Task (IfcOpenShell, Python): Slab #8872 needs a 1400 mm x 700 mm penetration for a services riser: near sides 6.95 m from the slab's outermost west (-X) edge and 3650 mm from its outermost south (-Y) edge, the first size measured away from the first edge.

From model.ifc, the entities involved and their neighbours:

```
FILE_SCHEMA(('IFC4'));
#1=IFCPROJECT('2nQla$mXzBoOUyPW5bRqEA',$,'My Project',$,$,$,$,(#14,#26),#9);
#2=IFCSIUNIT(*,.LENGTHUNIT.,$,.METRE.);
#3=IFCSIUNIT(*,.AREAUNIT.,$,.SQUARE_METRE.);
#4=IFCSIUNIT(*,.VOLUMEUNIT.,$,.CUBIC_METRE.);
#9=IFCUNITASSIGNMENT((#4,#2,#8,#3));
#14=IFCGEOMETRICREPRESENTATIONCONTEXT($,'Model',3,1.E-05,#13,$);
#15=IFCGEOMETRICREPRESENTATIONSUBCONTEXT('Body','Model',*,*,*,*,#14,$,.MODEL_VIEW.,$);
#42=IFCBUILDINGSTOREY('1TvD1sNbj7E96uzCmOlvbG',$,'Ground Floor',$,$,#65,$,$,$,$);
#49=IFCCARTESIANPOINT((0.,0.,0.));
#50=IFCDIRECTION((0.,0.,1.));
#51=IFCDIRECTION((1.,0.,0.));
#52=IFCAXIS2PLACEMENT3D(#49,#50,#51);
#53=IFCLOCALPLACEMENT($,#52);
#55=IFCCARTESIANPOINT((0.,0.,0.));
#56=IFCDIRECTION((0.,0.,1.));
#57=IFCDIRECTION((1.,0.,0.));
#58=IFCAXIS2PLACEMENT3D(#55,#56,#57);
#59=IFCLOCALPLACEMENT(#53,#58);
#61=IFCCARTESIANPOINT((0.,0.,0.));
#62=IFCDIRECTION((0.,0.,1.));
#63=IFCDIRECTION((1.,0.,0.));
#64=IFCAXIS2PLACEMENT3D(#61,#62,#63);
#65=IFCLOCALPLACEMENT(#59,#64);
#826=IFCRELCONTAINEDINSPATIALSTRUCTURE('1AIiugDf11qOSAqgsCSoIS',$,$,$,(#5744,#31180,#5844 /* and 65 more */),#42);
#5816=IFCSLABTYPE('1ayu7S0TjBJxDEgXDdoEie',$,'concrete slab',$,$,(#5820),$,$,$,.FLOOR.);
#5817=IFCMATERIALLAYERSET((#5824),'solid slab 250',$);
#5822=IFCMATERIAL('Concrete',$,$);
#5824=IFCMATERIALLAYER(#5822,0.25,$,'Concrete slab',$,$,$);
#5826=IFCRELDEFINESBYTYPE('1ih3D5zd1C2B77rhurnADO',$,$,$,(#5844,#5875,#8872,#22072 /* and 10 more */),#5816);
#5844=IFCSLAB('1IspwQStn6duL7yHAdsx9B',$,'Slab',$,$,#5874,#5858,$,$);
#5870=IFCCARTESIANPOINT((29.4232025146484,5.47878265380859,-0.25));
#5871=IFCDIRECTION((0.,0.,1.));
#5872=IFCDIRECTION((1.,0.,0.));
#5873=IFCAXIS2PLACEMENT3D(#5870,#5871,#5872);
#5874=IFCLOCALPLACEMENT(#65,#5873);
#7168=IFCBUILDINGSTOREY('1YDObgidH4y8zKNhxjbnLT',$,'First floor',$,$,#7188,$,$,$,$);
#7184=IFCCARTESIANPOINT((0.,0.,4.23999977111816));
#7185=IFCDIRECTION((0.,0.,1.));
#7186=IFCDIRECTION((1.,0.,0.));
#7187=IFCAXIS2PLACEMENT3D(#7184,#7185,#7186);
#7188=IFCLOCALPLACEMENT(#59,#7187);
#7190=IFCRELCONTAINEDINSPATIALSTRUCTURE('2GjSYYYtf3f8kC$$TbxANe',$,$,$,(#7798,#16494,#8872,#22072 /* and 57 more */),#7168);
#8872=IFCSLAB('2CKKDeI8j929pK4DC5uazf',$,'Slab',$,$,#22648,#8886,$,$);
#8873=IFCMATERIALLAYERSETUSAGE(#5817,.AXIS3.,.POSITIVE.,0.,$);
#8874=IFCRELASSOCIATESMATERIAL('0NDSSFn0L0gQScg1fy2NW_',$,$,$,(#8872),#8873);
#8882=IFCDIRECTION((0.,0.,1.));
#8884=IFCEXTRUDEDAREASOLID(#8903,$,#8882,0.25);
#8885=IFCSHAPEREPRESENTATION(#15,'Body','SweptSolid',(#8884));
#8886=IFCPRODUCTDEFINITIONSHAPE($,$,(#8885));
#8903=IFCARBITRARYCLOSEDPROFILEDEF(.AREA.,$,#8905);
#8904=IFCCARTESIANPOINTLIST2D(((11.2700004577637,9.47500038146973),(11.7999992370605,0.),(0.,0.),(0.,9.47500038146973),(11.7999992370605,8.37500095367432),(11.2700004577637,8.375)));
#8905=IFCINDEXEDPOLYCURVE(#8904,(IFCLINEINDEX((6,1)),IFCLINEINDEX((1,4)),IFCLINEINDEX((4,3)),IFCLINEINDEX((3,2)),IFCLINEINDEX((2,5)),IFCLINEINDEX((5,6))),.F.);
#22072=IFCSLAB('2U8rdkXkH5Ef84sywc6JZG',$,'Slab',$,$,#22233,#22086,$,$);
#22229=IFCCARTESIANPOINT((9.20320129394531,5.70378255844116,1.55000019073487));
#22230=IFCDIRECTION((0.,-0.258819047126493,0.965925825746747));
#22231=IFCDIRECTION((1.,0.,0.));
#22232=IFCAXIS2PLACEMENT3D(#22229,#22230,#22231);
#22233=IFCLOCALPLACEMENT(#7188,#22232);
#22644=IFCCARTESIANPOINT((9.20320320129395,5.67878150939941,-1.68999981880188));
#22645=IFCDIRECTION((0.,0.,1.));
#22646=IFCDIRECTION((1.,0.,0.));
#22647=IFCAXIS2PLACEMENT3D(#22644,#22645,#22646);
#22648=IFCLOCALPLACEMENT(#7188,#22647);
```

```python
import numpy as np
import ifcopenshell
import ifcopenshell.api.feature
import ifcopenshell.api.geometry
import ifcopenshell.api.root
import ifcopenshell.geom
import ifcopenshell.util.placement
import ifcopenshell.util.representation
import ifcopenshell.util.shape
import ifcopenshell.util.unit

model = ifcopenshell.open("model.ifc")
unit_scale = ifcopenshell.util.unit.calculate_unit_scale(model)
settings = ifcopenshell.geom.settings()


def volume(element):
    """Net volume in cubic metres, openings subtracted."""
    shape = ifcopenshell.geom.create_shape(settings, element)
    return ifcopenshell.util.shape.get_volume(shape.geometry)


slab = model.by_guid("2CKKDeI8j929pK4DC5uazf")
before = volume(slab)

# Extent in the slab's own axes, in metres. The edges named are its -X and -Y sides.
slab_shape = ifcopenshell.geom.create_shape(settings, slab)
vertices = ifcopenshell.util.shape.get_vertices(slab_shape.geometry)
x_min, y_min, bottom = vertices.min(axis=0)
top = vertices[:, 2].max()

opening = ifcopenshell.api.root.create_entity(model, ifc_class="IfcOpeningElement", name="Services riser opening", predefined_type="OPENING")
context = ifcopenshell.util.representation.get_context(model, "Model", "Body", "MODEL_VIEW")
width, depth = 1.4, 0.7
outline = [(0.0, 0.0), (width, 0.0), (width, depth), (0.0, depth), (0.0, 0.0)]
# Overshoot both faces by 50 mm so the cut is clean.
shape = ifcopenshell.api.geometry.add_slab_representation(
    model, context=context, depth=top - bottom + 0.1, polyline=outline
)
ifcopenshell.api.geometry.assign_representation(model, product=opening, representation=shape)

matrix = ifcopenshell.util.placement.get_local_placement(slab.ObjectPlacement)
matrix[:, 3] = matrix @ np.append(np.array([x_min + 6.95, y_min + 3.65, bottom - 0.05]) / unit_scale, 1.0)
ifcopenshell.api.geometry.edit_object_placement(model, product=opening, matrix=matrix, is_si=False)
ifcopenshell.api.feature.add_feature(model, feature=opening, element=slab)

after = volume(slab)

print(f"slab volume {before:.3f} -> {after:.3f} m3")

model.write("model_rev.ifc")
```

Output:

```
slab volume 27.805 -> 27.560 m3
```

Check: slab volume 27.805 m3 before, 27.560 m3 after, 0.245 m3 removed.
